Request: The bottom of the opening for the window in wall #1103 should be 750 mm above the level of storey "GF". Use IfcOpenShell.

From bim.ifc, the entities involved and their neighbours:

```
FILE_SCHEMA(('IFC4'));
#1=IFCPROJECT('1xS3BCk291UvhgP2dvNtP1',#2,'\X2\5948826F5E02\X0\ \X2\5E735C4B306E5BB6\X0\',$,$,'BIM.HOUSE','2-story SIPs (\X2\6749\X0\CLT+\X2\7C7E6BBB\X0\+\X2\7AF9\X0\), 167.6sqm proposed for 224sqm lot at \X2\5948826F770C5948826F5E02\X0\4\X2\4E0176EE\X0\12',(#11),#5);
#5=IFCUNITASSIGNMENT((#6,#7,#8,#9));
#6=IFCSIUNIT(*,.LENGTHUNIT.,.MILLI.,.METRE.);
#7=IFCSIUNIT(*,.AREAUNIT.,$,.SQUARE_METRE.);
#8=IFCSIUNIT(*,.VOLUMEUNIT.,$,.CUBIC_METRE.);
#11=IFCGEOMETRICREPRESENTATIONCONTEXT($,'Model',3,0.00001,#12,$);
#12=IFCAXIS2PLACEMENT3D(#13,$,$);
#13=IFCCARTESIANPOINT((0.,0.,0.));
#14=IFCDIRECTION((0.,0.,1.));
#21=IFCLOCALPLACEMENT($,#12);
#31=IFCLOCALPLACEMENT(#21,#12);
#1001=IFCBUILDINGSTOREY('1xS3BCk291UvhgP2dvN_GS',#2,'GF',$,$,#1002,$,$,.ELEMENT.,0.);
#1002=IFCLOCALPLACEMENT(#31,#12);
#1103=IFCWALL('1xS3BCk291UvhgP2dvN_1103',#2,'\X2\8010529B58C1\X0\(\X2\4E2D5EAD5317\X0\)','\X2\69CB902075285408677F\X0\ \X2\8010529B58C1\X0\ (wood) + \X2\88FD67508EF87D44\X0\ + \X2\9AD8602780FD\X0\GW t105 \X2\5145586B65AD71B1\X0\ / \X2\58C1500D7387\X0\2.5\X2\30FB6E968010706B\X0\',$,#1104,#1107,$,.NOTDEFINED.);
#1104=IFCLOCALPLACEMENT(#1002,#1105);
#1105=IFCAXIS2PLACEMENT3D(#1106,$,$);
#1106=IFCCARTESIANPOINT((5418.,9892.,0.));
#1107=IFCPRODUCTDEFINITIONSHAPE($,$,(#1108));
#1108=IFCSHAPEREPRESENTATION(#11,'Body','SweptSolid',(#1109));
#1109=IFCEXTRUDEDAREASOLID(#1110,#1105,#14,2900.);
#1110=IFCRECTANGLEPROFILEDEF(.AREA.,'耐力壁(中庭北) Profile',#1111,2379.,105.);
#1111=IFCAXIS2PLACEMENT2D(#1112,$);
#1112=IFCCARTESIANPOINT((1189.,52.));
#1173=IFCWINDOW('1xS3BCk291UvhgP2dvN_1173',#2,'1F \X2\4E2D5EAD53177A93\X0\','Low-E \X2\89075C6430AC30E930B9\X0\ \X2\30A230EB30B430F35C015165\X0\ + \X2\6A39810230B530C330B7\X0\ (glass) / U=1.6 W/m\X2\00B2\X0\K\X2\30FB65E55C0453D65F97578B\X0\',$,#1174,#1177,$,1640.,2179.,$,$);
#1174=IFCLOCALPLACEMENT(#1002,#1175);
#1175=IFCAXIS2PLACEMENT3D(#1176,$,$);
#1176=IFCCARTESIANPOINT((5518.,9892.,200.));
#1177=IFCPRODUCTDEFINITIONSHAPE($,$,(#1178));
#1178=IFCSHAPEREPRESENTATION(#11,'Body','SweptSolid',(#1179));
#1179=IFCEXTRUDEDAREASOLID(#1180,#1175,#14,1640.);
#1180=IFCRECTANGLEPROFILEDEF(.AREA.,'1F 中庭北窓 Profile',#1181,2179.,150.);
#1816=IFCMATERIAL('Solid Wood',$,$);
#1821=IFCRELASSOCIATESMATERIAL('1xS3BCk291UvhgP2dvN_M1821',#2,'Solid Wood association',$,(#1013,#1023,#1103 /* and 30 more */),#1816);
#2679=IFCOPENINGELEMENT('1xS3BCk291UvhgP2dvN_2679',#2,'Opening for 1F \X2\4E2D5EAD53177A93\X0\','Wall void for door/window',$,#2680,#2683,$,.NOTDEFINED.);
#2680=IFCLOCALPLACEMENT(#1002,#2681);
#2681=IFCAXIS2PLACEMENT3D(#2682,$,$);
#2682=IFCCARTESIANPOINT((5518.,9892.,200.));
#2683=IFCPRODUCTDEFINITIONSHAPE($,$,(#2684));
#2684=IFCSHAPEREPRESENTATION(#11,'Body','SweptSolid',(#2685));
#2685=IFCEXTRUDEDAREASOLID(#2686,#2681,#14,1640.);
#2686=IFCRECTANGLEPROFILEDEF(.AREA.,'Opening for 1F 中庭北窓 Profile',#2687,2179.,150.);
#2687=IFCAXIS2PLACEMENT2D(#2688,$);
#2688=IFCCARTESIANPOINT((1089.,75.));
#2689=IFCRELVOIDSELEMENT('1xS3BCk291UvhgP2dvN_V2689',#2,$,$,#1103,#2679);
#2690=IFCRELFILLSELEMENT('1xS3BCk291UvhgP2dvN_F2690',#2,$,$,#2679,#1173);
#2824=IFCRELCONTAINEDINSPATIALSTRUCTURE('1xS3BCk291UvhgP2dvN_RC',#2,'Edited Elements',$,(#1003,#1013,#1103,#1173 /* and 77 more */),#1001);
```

```python
import numpy as np
import ifcopenshell
import ifcopenshell.api.geometry
import ifcopenshell.geom
import ifcopenshell.util.element
import ifcopenshell.util.placement
import ifcopenshell.util.shape
import ifcopenshell.util.unit

model = ifcopenshell.open("bim.ifc")
unit_scale = ifcopenshell.util.unit.calculate_unit_scale(model)

window = model.by_guid("1xS3BCk291UvhgP2dvN_1173")
opening = window.FillsVoids[0].RelatingOpeningElement
storey = ifcopenshell.util.element.get_container(window, ifc_class="IfcBuildingStorey")
level = ifcopenshell.util.placement.get_local_placement(storey.ObjectPlacement)[2, 3]

# The opening's origin need not be at the sill, so measure its lowest point.
shape = ifcopenshell.geom.create_shape(ifcopenshell.geom.settings(), opening)
bottom = ifcopenshell.util.shape.get_shape_bottom_elevation(shape, shape.geometry) / unit_scale
dz = level + 0.75 / unit_scale - bottom

shift = np.array([0.0, 0.0, dz])
# The window is not placed relative to its opening, so move both.
for product in (opening, window):
    matrix = ifcopenshell.util.placement.get_local_placement(product.ObjectPlacement)
    matrix[:3, 3] += shift
    ifcopenshell.api.geometry.edit_object_placement(model, product=product, matrix=matrix, is_si=False)

print(f"moved by {dz * unit_scale:+.3f} m")

model.write("bim_edited.ifc")
```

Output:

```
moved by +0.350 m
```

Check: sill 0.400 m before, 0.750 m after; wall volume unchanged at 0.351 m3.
